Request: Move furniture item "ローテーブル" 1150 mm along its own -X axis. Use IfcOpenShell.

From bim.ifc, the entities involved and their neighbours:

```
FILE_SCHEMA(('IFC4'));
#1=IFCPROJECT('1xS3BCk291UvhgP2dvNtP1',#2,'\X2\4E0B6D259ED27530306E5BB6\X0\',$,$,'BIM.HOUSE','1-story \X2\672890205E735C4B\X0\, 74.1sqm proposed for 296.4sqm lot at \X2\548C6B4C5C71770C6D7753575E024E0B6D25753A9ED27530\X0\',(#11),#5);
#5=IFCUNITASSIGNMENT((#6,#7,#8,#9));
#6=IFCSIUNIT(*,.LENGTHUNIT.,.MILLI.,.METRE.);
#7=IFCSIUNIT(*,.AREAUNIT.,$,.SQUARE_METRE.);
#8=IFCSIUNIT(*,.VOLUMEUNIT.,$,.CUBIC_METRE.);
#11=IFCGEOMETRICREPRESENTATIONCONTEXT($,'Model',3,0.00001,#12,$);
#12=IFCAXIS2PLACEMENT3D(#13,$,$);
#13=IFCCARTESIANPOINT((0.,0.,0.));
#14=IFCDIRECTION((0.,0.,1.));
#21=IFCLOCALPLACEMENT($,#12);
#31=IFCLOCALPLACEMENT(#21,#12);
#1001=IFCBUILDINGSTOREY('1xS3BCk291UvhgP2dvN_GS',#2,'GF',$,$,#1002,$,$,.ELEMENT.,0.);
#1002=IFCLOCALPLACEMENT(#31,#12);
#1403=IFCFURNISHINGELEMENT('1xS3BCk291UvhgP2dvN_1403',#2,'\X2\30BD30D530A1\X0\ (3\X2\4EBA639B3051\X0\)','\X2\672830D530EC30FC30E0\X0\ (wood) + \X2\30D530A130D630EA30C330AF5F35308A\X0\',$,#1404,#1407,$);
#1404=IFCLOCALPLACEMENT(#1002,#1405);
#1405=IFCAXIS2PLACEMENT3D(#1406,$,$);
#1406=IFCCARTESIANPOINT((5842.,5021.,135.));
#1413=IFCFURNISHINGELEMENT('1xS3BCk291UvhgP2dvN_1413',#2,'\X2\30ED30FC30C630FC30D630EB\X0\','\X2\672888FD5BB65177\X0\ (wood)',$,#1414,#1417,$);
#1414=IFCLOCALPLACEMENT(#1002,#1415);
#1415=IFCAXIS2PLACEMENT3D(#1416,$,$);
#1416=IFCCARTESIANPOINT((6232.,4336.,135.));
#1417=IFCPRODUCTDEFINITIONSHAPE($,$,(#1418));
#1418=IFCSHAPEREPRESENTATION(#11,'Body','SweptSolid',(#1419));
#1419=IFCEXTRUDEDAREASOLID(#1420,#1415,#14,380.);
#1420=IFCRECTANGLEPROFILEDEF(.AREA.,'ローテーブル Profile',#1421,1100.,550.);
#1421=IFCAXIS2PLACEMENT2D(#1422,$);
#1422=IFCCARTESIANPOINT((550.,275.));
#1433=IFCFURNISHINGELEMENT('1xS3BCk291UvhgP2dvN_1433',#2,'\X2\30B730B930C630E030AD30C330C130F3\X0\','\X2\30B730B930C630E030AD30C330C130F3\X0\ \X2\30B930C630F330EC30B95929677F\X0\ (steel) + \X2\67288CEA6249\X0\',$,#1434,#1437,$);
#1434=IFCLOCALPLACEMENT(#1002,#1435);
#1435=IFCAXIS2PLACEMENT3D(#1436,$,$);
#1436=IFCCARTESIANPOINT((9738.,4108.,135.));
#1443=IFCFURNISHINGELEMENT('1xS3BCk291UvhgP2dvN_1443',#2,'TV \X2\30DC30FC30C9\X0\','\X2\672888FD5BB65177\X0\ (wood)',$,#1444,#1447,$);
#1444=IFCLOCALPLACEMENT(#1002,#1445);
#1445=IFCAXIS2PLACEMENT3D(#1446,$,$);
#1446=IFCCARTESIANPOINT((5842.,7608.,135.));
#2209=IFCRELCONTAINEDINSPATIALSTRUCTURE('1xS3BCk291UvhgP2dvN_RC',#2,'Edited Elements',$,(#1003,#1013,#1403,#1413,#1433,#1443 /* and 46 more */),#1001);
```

```python
import ifcopenshell
import ifcopenshell.api.geometry
import ifcopenshell.util.placement
import ifcopenshell.util.unit

model = ifcopenshell.open("bim.ifc")
unit_scale = ifcopenshell.util.unit.calculate_unit_scale(model)

item = model.by_guid("1xS3BCk291UvhgP2dvN_1413")
matrix = ifcopenshell.util.placement.get_local_placement(item.ObjectPlacement)
matrix[:3, 3] -= matrix[:3, 0] * 1.15 / unit_scale
ifcopenshell.api.geometry.edit_object_placement(model, product=item, matrix=matrix, is_si=False)

print(ifcopenshell.util.placement.get_local_placement(item.ObjectPlacement).round(3) + 0.0)

model.write("bim_updated.ifc")
```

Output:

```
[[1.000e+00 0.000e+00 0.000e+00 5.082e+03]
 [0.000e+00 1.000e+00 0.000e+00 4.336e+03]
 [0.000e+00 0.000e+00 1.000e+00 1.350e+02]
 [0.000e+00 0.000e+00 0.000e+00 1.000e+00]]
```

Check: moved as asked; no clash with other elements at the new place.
